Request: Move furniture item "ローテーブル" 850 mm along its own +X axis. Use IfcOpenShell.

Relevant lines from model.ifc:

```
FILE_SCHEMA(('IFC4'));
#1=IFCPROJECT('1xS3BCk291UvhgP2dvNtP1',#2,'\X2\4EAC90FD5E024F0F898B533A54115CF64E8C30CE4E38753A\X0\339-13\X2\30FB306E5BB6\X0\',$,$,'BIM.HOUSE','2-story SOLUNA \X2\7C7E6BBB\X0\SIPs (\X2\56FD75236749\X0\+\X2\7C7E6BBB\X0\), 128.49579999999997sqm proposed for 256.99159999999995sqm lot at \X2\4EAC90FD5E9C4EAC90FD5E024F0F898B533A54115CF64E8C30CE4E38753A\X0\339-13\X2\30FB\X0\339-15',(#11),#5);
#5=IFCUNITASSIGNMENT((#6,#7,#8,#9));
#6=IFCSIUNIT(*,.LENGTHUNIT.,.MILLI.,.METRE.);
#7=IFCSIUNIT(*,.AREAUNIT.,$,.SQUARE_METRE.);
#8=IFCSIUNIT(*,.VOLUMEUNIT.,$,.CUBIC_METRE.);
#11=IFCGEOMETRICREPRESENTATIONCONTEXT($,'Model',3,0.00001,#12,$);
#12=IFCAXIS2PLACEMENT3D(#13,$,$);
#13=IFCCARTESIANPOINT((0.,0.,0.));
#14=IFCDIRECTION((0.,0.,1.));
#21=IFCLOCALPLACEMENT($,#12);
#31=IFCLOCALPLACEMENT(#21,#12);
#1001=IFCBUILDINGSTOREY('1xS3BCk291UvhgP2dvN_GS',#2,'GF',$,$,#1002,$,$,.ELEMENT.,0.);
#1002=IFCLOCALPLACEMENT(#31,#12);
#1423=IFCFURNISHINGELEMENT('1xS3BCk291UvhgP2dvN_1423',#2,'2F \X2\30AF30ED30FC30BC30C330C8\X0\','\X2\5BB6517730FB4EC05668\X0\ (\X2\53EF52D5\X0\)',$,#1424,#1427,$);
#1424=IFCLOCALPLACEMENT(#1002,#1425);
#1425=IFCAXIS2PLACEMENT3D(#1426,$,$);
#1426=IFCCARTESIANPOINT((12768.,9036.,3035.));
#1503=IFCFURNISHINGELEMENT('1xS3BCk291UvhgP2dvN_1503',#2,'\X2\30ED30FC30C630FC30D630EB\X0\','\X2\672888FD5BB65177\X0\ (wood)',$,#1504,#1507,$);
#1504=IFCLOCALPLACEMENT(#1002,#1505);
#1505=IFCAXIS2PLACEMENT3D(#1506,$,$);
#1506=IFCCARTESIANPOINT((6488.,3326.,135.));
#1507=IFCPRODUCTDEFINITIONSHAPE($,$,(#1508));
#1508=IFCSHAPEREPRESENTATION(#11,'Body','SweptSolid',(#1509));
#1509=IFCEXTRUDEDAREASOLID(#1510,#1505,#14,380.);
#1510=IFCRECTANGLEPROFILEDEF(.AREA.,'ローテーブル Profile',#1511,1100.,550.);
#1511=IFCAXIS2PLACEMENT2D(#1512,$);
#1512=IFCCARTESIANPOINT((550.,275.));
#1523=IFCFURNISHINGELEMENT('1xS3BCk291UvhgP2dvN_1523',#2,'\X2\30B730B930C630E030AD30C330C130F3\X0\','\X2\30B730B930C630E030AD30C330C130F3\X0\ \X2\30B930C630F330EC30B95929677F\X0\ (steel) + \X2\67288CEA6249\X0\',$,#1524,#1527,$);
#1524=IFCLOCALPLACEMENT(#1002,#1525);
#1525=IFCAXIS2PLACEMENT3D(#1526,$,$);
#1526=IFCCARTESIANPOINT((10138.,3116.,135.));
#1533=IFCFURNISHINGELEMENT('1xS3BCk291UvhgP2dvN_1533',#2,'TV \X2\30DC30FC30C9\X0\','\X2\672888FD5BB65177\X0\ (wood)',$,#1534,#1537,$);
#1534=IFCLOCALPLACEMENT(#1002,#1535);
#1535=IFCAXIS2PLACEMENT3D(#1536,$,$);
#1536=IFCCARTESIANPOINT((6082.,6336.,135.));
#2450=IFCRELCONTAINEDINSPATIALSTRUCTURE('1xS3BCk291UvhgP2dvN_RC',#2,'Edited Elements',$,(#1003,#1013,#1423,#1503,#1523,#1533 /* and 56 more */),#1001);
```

```python
import ifcopenshell
import ifcopenshell.api.geometry
import ifcopenshell.util.placement

model = ifcopenshell.open("model.ifc")

item = model.by_guid("1xS3BCk291UvhgP2dvN_1503")
matrix = ifcopenshell.util.placement.get_local_placement(item.ObjectPlacement)
matrix[:3, 3] += matrix[:3, 0] * 850.0
ifcopenshell.api.geometry.edit_object_placement(model, product=item, matrix=matrix, is_si=False)

print(ifcopenshell.util.placement.get_local_placement(item.ObjectPlacement).round(3) + 0.0)

model.write("model_edited.ifc")
```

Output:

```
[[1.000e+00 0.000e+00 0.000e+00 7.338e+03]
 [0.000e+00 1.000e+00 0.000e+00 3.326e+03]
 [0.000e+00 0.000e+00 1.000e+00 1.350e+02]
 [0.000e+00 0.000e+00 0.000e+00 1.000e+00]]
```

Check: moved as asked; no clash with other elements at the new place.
